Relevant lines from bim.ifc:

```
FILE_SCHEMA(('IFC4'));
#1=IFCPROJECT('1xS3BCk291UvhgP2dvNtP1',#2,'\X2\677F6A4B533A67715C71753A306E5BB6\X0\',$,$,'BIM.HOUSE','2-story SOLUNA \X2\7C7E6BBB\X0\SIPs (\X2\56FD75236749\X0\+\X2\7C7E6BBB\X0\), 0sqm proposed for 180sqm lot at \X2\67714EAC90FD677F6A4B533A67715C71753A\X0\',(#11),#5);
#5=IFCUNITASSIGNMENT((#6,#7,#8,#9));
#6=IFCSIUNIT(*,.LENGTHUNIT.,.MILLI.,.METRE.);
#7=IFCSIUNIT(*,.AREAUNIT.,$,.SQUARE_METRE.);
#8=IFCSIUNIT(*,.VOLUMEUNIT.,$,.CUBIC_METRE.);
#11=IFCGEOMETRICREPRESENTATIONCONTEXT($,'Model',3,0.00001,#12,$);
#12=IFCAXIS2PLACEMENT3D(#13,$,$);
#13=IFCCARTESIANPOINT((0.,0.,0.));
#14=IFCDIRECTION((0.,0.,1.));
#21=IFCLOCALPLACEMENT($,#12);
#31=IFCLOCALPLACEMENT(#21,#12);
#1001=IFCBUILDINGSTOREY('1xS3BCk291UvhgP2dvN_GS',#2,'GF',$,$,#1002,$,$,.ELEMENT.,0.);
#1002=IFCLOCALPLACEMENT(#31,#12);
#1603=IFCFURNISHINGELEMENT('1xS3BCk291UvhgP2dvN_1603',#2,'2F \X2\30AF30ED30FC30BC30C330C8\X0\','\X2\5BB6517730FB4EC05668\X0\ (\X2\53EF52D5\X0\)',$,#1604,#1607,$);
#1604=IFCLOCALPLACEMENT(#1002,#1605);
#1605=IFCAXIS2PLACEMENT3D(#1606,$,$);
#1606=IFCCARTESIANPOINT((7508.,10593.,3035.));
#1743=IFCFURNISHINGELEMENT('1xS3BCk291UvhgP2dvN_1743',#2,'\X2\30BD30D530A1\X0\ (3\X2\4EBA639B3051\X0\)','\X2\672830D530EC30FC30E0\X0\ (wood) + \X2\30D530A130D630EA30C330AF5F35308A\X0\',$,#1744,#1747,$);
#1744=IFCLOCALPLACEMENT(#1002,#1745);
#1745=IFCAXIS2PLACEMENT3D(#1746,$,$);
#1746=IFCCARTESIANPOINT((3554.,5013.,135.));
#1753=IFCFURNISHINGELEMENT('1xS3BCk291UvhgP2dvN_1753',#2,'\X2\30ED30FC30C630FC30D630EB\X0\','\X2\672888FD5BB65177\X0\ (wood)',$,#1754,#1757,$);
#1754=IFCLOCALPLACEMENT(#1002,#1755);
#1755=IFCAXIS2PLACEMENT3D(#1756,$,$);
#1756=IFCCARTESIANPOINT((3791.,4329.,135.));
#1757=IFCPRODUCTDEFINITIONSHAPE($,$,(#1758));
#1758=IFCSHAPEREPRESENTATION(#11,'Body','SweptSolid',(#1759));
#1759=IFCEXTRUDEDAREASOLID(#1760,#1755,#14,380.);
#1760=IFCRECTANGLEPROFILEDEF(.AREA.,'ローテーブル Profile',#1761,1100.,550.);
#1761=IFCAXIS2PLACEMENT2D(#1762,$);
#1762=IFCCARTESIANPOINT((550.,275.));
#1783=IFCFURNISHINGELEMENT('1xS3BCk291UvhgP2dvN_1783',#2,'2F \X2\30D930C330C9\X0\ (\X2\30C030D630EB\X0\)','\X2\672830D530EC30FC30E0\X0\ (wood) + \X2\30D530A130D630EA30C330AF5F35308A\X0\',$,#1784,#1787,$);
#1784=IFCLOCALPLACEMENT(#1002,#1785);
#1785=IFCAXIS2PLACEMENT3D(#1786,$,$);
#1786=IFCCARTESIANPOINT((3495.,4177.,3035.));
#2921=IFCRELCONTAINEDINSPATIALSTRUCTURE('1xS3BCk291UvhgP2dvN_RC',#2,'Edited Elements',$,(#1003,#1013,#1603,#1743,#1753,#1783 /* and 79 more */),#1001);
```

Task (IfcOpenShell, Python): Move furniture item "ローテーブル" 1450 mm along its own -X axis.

```python
import ifcopenshell
import ifcopenshell.api.geometry
import ifcopenshell.util.placement

model = ifcopenshell.open("bim.ifc")

item = model.by_guid("1xS3BCk291UvhgP2dvN_1753")
matrix = ifcopenshell.util.placement.get_local_placement(item.ObjectPlacement)
matrix[:3, 3] -= matrix[:3, 0] * 1450.0
ifcopenshell.api.geometry.edit_object_placement(model, product=item, matrix=matrix, is_si=False)

print(ifcopenshell.util.placement.get_local_placement(item.ObjectPlacement).round(3) + 0.0)

model.write("bim_v2.ifc")
```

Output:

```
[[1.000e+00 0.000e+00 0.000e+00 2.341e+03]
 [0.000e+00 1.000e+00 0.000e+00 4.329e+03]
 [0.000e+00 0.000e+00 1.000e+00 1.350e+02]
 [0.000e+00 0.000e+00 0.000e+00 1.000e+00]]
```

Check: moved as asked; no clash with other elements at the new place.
